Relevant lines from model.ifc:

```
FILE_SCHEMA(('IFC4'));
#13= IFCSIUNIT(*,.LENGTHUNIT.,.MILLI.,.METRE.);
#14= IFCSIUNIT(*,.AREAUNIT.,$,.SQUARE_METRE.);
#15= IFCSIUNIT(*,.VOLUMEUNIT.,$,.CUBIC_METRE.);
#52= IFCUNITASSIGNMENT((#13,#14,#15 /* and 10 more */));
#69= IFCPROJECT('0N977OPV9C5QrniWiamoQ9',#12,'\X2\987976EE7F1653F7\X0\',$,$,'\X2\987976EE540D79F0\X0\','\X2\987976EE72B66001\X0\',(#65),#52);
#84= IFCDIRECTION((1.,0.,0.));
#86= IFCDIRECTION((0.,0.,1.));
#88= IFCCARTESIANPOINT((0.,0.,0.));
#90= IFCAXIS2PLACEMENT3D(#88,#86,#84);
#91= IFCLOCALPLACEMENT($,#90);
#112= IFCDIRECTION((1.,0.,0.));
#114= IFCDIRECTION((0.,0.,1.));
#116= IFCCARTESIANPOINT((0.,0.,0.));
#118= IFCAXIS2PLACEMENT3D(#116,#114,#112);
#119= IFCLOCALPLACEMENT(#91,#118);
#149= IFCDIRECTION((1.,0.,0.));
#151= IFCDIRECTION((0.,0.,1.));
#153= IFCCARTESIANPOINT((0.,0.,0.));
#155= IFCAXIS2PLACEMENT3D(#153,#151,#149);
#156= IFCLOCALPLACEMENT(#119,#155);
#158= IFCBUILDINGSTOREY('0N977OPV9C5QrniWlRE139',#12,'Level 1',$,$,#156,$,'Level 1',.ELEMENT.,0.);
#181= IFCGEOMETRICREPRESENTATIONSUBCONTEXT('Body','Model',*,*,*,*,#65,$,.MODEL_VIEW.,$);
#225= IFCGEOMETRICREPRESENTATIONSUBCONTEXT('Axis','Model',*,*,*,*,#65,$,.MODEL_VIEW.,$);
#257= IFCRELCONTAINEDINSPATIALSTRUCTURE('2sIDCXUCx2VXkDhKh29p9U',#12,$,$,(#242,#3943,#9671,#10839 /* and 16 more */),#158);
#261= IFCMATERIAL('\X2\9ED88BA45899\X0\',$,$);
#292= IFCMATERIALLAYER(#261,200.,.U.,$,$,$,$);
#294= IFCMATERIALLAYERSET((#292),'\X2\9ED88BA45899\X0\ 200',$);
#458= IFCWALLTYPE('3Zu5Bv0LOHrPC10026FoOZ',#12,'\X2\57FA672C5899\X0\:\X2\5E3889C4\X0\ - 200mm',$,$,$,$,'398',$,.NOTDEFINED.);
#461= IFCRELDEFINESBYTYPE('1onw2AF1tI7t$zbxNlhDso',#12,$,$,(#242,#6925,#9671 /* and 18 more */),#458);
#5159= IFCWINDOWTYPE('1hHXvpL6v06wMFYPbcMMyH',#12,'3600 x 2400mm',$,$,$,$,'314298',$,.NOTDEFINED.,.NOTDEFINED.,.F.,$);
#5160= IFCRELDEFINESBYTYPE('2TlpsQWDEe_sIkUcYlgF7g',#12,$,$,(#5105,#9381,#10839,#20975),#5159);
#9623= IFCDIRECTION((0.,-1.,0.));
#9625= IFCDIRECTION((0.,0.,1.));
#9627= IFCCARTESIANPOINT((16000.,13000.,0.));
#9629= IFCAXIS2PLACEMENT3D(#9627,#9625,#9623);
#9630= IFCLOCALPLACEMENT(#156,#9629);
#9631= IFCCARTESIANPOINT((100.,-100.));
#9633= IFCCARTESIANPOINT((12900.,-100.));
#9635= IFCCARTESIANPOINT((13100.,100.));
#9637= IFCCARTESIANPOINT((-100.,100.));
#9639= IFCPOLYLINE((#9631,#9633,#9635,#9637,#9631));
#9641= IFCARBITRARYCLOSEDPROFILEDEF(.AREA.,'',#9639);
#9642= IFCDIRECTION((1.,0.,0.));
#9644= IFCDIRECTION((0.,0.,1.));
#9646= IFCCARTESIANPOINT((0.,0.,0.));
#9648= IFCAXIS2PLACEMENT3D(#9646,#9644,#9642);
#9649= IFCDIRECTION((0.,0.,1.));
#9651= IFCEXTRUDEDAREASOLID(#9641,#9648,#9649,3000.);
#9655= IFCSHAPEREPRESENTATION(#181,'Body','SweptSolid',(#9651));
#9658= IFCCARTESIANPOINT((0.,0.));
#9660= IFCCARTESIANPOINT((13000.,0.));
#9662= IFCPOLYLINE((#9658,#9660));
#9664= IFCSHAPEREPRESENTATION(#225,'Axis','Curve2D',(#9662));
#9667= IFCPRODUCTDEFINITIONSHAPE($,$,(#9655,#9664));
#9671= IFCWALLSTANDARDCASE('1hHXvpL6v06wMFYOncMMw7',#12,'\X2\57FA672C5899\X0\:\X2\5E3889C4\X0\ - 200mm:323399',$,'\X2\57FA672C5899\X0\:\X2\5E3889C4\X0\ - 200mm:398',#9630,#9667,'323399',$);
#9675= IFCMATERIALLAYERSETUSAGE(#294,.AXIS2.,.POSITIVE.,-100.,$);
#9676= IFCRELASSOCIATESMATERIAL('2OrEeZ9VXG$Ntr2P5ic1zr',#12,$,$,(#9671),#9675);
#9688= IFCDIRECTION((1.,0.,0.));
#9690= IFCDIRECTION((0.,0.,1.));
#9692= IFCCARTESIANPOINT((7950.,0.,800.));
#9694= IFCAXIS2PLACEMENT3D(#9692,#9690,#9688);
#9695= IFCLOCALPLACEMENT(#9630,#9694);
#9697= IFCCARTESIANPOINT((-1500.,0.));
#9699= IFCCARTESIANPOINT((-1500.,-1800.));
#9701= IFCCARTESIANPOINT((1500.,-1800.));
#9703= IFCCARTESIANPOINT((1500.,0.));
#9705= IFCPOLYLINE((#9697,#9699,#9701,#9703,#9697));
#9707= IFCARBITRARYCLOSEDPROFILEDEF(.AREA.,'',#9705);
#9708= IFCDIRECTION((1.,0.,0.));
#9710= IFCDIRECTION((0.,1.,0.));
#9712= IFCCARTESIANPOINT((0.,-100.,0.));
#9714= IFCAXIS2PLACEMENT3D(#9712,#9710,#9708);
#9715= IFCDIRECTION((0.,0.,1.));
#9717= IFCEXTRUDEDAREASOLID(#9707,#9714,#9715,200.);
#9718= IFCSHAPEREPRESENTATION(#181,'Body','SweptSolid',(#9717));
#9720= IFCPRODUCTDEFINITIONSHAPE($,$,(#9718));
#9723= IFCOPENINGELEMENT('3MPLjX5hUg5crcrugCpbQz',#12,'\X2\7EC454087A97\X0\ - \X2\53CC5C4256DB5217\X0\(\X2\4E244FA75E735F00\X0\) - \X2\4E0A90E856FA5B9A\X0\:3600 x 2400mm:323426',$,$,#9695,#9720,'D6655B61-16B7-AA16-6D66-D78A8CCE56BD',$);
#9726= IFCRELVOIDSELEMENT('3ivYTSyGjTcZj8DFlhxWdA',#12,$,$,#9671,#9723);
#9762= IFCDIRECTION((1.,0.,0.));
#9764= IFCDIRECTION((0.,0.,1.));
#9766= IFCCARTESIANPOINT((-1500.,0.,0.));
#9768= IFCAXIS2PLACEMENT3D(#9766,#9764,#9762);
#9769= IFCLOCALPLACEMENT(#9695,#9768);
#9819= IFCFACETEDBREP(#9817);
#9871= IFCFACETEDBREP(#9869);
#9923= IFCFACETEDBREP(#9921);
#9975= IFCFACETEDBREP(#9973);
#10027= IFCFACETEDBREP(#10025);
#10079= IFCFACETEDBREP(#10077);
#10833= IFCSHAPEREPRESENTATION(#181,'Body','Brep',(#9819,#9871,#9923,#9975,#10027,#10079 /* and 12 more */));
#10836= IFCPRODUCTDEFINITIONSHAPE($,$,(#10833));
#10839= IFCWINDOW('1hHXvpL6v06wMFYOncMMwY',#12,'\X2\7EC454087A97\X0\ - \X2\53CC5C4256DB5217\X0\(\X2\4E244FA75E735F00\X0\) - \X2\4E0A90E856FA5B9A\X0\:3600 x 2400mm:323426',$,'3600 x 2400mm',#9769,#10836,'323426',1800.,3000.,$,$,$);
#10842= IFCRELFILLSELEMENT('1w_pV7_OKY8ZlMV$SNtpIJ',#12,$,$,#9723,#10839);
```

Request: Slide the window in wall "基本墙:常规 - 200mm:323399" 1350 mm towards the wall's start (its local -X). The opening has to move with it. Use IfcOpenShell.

```python
import ifcopenshell
import ifcopenshell.api.geometry
import ifcopenshell.util.placement
import ifcopenshell.util.unit

model = ifcopenshell.open("model.ifc")
unit_scale = ifcopenshell.util.unit.calculate_unit_scale(model)

window = model.by_guid("1hHXvpL6v06wMFYOncMMwY")
opening = window.FillsVoids[0].RelatingOpeningElement
wall = opening.VoidsElements[0].RelatingBuildingElement

wall_matrix = ifcopenshell.util.placement.get_local_placement(wall.ObjectPlacement)
shift = wall_matrix[:3, 0] * -1.35 / unit_scale
before = ifcopenshell.util.placement.get_local_placement(window.ObjectPlacement)[:3, 3].copy()

# The window is placed relative to its opening, so it follows when the opening moves.
matrix = ifcopenshell.util.placement.get_local_placement(opening.ObjectPlacement)
matrix[:3, 3] += shift
ifcopenshell.api.geometry.edit_object_placement(
    model, product=opening, matrix=matrix, is_si=False, should_transform_children=True
)

after = ifcopenshell.util.placement.get_local_placement(window.ObjectPlacement)[:3, 3]
print("window moved by", (after - before).round(3) + 0.0)

model.write("model_rev.ifc")
```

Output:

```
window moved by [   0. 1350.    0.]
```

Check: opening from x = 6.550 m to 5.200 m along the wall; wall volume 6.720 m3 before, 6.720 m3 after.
